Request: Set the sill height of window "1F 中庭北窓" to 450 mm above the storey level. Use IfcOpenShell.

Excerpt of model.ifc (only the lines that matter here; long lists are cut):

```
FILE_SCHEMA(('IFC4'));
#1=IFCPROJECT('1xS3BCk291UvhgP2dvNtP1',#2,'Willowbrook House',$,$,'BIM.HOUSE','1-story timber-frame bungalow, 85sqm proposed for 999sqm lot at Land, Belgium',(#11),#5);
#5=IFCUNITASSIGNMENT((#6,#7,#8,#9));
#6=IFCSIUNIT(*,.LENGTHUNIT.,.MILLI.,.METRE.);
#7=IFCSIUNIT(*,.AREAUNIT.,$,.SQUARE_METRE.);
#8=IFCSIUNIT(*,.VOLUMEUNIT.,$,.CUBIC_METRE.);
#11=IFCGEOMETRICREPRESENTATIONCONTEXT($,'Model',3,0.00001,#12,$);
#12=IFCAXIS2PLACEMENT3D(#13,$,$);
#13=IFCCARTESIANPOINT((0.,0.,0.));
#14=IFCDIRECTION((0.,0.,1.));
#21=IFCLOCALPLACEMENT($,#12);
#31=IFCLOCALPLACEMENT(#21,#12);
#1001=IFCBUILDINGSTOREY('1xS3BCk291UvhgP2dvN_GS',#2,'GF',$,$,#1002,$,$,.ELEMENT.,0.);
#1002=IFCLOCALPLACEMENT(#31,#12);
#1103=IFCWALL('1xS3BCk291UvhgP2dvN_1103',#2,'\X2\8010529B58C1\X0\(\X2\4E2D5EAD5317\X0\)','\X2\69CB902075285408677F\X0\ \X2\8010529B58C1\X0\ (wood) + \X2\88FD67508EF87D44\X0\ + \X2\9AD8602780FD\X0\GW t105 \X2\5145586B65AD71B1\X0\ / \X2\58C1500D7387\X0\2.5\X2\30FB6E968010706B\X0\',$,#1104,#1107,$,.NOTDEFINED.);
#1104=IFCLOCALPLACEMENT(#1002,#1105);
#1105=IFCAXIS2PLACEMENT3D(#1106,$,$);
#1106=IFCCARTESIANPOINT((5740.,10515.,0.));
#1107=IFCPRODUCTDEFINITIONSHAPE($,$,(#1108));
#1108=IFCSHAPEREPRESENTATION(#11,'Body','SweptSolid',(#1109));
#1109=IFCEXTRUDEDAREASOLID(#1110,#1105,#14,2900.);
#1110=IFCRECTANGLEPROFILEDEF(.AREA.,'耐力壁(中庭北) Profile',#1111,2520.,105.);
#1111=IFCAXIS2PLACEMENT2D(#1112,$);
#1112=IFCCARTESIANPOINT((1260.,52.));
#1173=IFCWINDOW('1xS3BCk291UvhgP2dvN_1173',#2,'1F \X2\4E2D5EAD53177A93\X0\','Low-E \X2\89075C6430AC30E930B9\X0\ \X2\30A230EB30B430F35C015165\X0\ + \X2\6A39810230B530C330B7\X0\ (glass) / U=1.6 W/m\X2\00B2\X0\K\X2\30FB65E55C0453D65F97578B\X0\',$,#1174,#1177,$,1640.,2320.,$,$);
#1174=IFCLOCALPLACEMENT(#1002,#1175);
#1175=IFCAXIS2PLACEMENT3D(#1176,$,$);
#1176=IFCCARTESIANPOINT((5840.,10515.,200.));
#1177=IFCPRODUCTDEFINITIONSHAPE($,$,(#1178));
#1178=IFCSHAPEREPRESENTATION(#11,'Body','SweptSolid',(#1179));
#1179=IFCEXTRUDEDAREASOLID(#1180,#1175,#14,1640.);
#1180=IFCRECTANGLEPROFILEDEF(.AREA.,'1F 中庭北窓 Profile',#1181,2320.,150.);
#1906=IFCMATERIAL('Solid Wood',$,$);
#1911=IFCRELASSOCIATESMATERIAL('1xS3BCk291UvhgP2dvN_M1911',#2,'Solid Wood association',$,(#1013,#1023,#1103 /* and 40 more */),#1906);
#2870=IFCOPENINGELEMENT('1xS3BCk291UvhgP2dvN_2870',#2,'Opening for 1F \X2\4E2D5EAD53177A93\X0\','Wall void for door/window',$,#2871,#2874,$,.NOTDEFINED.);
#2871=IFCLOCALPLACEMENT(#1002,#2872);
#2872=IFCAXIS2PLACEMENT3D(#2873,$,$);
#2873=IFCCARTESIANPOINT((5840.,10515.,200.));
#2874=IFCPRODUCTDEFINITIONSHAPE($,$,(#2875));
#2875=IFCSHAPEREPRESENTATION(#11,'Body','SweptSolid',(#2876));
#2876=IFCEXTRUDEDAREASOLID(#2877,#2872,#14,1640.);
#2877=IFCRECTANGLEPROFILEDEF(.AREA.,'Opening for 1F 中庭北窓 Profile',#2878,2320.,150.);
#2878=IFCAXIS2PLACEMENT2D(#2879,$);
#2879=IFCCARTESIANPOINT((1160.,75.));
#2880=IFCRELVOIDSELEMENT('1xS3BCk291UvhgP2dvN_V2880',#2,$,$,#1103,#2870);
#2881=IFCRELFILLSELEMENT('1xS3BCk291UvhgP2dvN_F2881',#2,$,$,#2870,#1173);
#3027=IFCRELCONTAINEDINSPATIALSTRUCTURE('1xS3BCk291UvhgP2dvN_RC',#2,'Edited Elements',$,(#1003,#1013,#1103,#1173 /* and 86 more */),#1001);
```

```python
import numpy as np
import ifcopenshell
import ifcopenshell.api.geometry
import ifcopenshell.geom
import ifcopenshell.util.element
import ifcopenshell.util.placement
import ifcopenshell.util.shape
import ifcopenshell.util.unit

model = ifcopenshell.open("model.ifc")
unit_scale = ifcopenshell.util.unit.calculate_unit_scale(model)

window = model.by_guid("1xS3BCk291UvhgP2dvN_1173")
opening = window.FillsVoids[0].RelatingOpeningElement
storey = ifcopenshell.util.element.get_container(window, ifc_class="IfcBuildingStorey")
level = ifcopenshell.util.placement.get_local_placement(storey.ObjectPlacement)[2, 3]

# The opening's origin need not be at the sill, so measure its lowest point.
shape = ifcopenshell.geom.create_shape(ifcopenshell.geom.settings(), opening)
bottom = ifcopenshell.util.shape.get_shape_bottom_elevation(shape, shape.geometry) / unit_scale
dz = level + 0.45 / unit_scale - bottom

shift = np.array([0.0, 0.0, dz])
# The window is not placed relative to its opening, so move both.
for product in (opening, window):
    matrix = ifcopenshell.util.placement.get_local_placement(product.ObjectPlacement)
    matrix[:3, 3] += shift
    ifcopenshell.api.geometry.edit_object_placement(model, product=product, matrix=matrix, is_si=False)

print(f"moved by {dz * unit_scale:+.3f} m")

model.write("model_updated.ifc")
```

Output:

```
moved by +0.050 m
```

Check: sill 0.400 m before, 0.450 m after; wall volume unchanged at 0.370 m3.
